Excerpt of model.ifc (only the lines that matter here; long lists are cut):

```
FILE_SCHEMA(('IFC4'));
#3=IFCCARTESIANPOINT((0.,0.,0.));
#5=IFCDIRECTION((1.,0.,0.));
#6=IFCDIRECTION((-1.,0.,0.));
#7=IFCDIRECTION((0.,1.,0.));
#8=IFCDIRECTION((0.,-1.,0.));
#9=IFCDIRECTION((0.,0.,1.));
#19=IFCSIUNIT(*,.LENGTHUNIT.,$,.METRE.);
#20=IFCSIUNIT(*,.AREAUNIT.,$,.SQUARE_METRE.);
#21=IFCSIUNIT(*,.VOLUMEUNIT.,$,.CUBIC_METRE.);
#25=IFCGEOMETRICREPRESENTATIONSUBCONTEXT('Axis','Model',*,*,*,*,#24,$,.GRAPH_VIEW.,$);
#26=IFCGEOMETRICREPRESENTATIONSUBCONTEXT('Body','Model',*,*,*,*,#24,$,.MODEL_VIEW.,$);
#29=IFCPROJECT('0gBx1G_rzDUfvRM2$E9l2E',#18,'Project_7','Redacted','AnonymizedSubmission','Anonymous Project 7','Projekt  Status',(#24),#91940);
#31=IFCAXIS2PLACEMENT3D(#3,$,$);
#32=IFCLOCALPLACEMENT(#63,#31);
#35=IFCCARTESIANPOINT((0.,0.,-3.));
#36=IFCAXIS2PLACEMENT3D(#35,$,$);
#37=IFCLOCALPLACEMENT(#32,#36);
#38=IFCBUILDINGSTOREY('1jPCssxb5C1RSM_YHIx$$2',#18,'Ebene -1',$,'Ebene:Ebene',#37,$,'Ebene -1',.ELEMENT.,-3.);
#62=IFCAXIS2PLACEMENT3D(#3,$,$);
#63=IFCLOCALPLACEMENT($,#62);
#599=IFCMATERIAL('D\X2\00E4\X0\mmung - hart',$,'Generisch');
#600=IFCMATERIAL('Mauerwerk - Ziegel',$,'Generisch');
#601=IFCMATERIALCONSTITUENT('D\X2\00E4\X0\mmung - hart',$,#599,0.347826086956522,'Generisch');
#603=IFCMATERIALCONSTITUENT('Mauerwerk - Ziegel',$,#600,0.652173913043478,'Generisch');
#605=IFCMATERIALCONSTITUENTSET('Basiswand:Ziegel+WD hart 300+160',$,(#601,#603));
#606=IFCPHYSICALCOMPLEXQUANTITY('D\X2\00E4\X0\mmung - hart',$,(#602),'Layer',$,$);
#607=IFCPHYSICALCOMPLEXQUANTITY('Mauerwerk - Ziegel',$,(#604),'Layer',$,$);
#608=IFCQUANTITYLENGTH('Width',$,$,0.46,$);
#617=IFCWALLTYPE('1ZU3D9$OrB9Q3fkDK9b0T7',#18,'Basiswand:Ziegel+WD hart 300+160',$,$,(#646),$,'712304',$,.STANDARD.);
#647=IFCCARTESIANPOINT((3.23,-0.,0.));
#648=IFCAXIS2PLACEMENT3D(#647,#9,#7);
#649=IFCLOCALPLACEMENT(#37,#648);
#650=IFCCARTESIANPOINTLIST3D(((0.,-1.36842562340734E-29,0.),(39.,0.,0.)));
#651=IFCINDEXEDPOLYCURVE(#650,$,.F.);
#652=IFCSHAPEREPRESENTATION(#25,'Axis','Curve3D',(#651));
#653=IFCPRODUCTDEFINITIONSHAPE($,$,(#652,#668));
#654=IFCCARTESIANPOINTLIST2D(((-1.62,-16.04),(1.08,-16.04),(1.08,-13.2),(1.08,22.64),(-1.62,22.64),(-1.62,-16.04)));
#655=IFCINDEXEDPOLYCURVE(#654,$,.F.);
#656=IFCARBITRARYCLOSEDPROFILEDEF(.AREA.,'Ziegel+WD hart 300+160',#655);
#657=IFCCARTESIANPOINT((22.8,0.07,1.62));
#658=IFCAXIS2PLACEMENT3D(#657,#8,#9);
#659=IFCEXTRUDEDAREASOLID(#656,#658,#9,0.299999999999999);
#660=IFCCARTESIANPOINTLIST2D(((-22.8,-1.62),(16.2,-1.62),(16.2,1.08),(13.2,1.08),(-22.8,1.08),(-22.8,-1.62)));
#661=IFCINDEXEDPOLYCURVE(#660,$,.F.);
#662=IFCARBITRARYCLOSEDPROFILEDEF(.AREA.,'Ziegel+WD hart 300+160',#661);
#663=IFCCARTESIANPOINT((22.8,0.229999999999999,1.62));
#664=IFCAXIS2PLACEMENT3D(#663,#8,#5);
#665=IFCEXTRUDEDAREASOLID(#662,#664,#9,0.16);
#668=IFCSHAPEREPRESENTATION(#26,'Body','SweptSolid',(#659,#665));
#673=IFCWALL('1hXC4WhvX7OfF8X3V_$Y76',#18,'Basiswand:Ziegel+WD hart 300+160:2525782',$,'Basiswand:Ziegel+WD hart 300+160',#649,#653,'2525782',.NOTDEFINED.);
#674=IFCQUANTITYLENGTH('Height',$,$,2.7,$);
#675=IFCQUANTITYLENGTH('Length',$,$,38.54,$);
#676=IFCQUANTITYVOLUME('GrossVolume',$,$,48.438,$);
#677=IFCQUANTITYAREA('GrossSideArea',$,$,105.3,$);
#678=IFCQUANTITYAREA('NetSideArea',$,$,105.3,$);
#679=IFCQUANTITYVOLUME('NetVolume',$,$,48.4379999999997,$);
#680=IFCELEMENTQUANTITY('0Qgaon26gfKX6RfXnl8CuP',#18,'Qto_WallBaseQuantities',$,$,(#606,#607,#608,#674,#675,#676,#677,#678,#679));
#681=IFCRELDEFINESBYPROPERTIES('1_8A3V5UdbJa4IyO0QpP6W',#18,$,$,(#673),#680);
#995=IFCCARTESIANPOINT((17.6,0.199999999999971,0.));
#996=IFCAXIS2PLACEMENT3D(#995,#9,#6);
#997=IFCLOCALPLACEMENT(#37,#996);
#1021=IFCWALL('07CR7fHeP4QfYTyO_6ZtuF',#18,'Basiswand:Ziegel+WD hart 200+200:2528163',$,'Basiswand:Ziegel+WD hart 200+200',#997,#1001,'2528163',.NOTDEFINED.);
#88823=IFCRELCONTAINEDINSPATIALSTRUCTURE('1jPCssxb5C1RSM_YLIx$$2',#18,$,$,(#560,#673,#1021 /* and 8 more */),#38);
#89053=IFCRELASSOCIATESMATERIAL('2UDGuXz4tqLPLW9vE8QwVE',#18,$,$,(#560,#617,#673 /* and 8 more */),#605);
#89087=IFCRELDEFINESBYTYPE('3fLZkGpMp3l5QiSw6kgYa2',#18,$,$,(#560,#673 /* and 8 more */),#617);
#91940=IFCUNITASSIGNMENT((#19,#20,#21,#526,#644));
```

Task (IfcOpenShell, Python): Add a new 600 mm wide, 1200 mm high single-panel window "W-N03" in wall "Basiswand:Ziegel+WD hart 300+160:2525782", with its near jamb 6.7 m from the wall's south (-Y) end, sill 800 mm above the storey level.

```python
import numpy as np
import ifcopenshell
import ifcopenshell.api.feature
import ifcopenshell.api.geometry
import ifcopenshell.api.pset
import ifcopenshell.api.root
import ifcopenshell.api.spatial
import ifcopenshell.geom
import ifcopenshell.util.element
import ifcopenshell.util.placement
import ifcopenshell.util.representation
import ifcopenshell.util.shape
import ifcopenshell.util.unit

model = ifcopenshell.open("model.ifc")
unit_scale = ifcopenshell.util.unit.calculate_unit_scale(model)
area_scale = ifcopenshell.util.unit.calculate_unit_scale(model, "AREAUNIT")
volume_scale = ifcopenshell.util.unit.calculate_unit_scale(model, "VOLUMEUNIT")
settings = ifcopenshell.geom.settings()


def volume(element):
    """Net volume in cubic metres, openings subtracted."""
    shape = ifcopenshell.geom.create_shape(settings, element)
    return ifcopenshell.util.shape.get_volume(shape.geometry)


wall = model.by_id(673)
storey = ifcopenshell.util.element.get_container(wall, ifc_class="IfcBuildingStorey")
context = ifcopenshell.util.representation.get_context(model, "Model", "Body", "MODEL_VIEW")
before = volume(wall)

width, height, from_end, sill = 0.6, 1.2, 6.7, 0.8  # metres

# The wall runs along its own X axis, and the end named is its -X end.
wall_shape = ifcopenshell.geom.create_shape(settings, wall)
x, y, z = ifcopenshell.util.shape.get_vertices(wall_shape.geometry).T
start = x.min() + from_end
face, thickness = float(y.min()), float(y.max() - y.min())
wall_matrix = ifcopenshell.util.placement.get_local_placement(wall.ObjectPlacement)
level = ifcopenshell.util.placement.get_local_placement(storey.ObjectPlacement)[2, 3]


def in_wall(x, y):
    """Placement at x, y metres in the wall's axes, at sill height."""
    matrix = wall_matrix.copy()
    matrix[:, 3] = wall_matrix @ np.array([x / unit_scale, y / unit_scale, 0.0, 1.0])
    matrix[2, 3] = level + sill / unit_scale
    return matrix


# Opening: a box that overshoots both wall faces by 50 mm.
opening = ifcopenshell.api.root.create_entity(model, ifc_class="IfcOpeningElement", predefined_type="OPENING")
box = ifcopenshell.api.geometry.add_wall_representation(
    model, context=context, length=width, height=height, thickness=thickness + 0.1
)
ifcopenshell.api.geometry.assign_representation(model, product=opening, representation=box)
ifcopenshell.api.geometry.edit_object_placement(model, product=opening, matrix=in_wall(start, face - 0.05), is_si=False)
ifcopenshell.api.feature.add_feature(model, feature=opening, element=wall)

window = ifcopenshell.api.root.create_entity(model, ifc_class="IfcWindow", name="W-N03", predefined_type="WINDOW")
window.OverallWidth, window.OverallHeight = width / unit_scale, height / unit_scale
window.PartitioningType = "SINGLE_PANEL"
body = ifcopenshell.api.geometry.add_window_representation(
    model,
    context=context,
    overall_width=window.OverallWidth,
    overall_height=window.OverallHeight,
    partition_type="SINGLE_PANEL",
)
ifcopenshell.api.geometry.assign_representation(model, product=window, representation=body)
ifcopenshell.api.spatial.assign_container(model, products=[window], relating_structure=storey)
ifcopenshell.api.feature.add_filling(model, opening=opening, element=window)

# Centre the window in the wall's thickness.
ifcopenshell.api.geometry.edit_object_placement(model, product=window, matrix=in_wall(start, face), is_si=False)
window_shape = ifcopenshell.geom.create_shape(settings, window)
depth = ifcopenshell.util.shape.get_vertices(window_shape.geometry)[:, 1]
offset = face + thickness / 2 - (depth.min() + depth.max()) / 2
ifcopenshell.api.geometry.edit_object_placement(model, product=window, matrix=in_wall(start, offset), is_si=False)

after = volume(wall)

# Update the wall's stored quantities.
qto = model.by_id(ifcopenshell.util.element.get_pset(wall, "Qto_WallBaseQuantities", should_inherit=False)["id"])
ifcopenshell.api.pset.edit_qto(model, qto=qto, properties={
    "NetSideArea": after / thickness / area_scale,
    "NetVolume": after / volume_scale,
})

print(f"wall volume {before:.3f} -> {after:.3f} m3")

model.write("model_updated.ifc")
```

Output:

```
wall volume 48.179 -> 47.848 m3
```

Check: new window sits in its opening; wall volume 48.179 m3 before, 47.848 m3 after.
